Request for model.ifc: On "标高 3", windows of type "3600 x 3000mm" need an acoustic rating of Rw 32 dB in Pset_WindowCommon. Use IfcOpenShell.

First a look at what the model holds.

```python
import ifcopenshell
import ifcopenshell.util.element

model = ifcopenshell.open("model.ifc")
print(model.schema)
storey = next(s for s in model.by_type("IfcBuildingStorey") if s.Name == "标高 3")
windows = [e for e in ifcopenshell.util.element.get_decomposition(storey) if e.is_a("IfcWindow")]
seen = {}
for e in windows:
    element_type = ifcopenshell.util.element.get_type(e)
    key = (element_type.Name if element_type != e and element_type else None, ifcopenshell.util.element.get_pset(e, "Pset_WindowCommon", "AcousticRating"))
    seen[key] = seen.get(key, 0) + 1
for (name, value), count in sorted(seen.items(), key=str):
    print(count, "x", name, "|", value)
```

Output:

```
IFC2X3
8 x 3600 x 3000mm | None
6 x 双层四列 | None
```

```python
import ifcopenshell
import ifcopenshell.api.pset
import ifcopenshell.util.element

model = ifcopenshell.open("model.ifc")

storey = next(s for s in model.by_type("IfcBuildingStorey") if s.Name == "标高 3")
windows = [e for e in ifcopenshell.util.element.get_decomposition(storey) if e.is_a("IfcWindow")]

count = 0
for e in windows:
    element_type = ifcopenshell.util.element.get_type(e)
    if element_type in (None, e) or element_type.Name != "3600 x 3000mm":
        continue
    # add_pset returns the element's existing set when there is one.
    pset = ifcopenshell.api.pset.add_pset(model, product=e, name="Pset_WindowCommon")
    ifcopenshell.api.pset.edit_pset(model, pset=pset, properties={"AcousticRating": "Rw 32 dB"})
    count += 1

print(count, "windows updated")

model.write("model_updated.ifc")
```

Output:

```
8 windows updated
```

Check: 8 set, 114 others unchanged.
